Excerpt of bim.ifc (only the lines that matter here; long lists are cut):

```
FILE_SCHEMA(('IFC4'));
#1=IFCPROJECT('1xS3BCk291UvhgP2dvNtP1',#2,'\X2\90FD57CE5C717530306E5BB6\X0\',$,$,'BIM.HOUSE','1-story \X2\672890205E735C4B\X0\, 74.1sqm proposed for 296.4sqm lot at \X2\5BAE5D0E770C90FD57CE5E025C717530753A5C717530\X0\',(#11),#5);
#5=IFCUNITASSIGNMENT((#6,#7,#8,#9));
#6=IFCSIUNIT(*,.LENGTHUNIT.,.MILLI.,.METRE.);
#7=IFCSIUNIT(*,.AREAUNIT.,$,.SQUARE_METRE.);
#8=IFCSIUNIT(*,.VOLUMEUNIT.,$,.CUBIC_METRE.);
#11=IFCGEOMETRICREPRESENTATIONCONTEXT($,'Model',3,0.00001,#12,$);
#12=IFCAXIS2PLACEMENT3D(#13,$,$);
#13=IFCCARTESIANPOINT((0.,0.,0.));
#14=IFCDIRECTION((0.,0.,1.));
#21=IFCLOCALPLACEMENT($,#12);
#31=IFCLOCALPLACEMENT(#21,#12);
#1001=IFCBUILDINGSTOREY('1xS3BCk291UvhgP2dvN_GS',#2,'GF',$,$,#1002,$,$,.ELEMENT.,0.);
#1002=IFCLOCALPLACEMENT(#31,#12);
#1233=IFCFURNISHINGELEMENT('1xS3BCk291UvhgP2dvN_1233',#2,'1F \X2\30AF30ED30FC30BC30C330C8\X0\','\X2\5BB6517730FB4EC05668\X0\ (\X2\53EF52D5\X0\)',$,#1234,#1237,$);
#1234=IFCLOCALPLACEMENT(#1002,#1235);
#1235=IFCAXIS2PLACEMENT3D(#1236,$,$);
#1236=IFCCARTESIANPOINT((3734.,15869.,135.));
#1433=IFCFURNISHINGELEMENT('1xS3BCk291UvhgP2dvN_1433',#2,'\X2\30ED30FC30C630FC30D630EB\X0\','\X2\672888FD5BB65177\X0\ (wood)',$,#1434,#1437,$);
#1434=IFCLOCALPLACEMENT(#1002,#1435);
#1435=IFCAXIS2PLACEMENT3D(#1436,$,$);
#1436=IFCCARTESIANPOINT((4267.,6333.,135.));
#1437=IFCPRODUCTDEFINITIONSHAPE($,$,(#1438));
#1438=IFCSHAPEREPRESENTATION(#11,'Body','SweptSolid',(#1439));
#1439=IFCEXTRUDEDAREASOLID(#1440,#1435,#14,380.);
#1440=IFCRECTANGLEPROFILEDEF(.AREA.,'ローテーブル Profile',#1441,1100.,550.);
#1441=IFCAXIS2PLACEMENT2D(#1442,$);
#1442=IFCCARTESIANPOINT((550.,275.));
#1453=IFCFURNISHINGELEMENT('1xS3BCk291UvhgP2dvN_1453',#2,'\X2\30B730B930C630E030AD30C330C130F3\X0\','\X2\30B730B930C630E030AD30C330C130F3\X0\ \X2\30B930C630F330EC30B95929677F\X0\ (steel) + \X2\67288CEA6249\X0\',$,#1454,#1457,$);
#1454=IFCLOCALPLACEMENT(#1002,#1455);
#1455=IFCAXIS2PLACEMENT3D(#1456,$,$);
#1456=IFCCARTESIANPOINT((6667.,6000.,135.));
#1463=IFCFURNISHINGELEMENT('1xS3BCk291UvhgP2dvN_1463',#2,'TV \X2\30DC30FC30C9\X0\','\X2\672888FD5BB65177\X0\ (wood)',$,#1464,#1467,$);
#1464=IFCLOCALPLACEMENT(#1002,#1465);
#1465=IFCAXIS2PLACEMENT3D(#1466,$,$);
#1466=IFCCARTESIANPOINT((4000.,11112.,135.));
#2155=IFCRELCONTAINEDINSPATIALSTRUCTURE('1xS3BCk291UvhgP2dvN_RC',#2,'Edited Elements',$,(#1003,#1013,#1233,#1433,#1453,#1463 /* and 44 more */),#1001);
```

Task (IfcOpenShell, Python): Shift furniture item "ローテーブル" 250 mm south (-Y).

```python
import ifcopenshell
import ifcopenshell.api.geometry
import ifcopenshell.util.placement
import ifcopenshell.util.unit

model = ifcopenshell.open("bim.ifc")
unit_scale = ifcopenshell.util.unit.calculate_unit_scale(model)

item = model.by_guid("1xS3BCk291UvhgP2dvN_1433")
matrix = ifcopenshell.util.placement.get_local_placement(item.ObjectPlacement)
matrix[1, 3] -= 0.25 / unit_scale
ifcopenshell.api.geometry.edit_object_placement(model, product=item, matrix=matrix, is_si=False)

print(ifcopenshell.util.placement.get_local_placement(item.ObjectPlacement).round(3) + 0.0)

model.write("bim_updated.ifc")
```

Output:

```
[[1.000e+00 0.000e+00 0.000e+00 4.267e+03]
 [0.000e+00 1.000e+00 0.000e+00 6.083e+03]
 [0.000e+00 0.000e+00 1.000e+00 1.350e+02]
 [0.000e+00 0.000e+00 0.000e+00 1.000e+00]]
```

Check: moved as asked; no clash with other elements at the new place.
